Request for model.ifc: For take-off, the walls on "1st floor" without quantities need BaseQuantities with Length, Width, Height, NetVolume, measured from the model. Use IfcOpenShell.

First a look at what the model holds.

```python
import ifcopenshell
import ifcopenshell.util.element
import ifcopenshell.util.unit

model = ifcopenshell.open("model.ifc")
print(model.schema)
for unit_type in ("LENGTHUNIT", "AREAUNIT", "VOLUMEUNIT"):
    print(unit_type, ifcopenshell.util.unit.calculate_unit_scale(model, unit_type))
storey = next(s for s in model.by_type("IfcBuildingStorey") if s.Name == "1st floor")
walls = [e for e in ifcopenshell.util.element.get_decomposition(storey) if e.is_a("IfcWall")]
for e in sorted(walls, key=lambda e: e.id()):
    print(e.id(), e.is_a(), e.Name, list(ifcopenshell.util.element.get_psets(e, qtos_only=True)), sep=" | ")
```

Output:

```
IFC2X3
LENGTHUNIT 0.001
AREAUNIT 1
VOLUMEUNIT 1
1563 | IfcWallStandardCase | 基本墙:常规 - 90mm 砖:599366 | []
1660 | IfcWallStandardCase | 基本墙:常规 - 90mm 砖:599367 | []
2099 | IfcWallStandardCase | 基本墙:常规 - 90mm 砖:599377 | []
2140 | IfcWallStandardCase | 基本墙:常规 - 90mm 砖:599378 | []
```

```python
import ifcopenshell
import ifcopenshell.api.pset
import ifcopenshell.geom
import ifcopenshell.util.element
import ifcopenshell.util.shape
import ifcopenshell.util.unit

model = ifcopenshell.open("model.ifc")
unit_scale = ifcopenshell.util.unit.calculate_unit_scale(model)
volume_scale = ifcopenshell.util.unit.calculate_unit_scale(model, "VOLUMEUNIT")
settings = ifcopenshell.geom.settings()

storey = next(s for s in model.by_type("IfcBuildingStorey") if s.Name == "1st floor")
walls = [e for e in ifcopenshell.util.element.get_decomposition(storey) if e.is_a("IfcWall")]

for e in sorted(walls, key=lambda e: e.id()):
    if ifcopenshell.util.element.get_psets(e, qtos_only=True, should_inherit=False):
        continue
    # Geometry comes back in metres, in the element's own axes.
    shape = ifcopenshell.geom.create_shape(settings, e)
    values = {
        "Length": ifcopenshell.util.shape.get_x(shape.geometry) / unit_scale,
        "Width": ifcopenshell.util.shape.get_y(shape.geometry) / unit_scale,
        "Height": ifcopenshell.util.shape.get_z(shape.geometry) / unit_scale,
        "NetVolume": ifcopenshell.util.shape.get_volume(shape.geometry) / volume_scale,
    }
    qto = ifcopenshell.api.pset.add_qto(model, product=e, name="BaseQuantities")
    ifcopenshell.api.pset.edit_qto(model, qto=qto, properties=values)
    print(e.id(), {k: round(v, 3) for k, v in values.items()})

model.write("model_edited.ifc")
```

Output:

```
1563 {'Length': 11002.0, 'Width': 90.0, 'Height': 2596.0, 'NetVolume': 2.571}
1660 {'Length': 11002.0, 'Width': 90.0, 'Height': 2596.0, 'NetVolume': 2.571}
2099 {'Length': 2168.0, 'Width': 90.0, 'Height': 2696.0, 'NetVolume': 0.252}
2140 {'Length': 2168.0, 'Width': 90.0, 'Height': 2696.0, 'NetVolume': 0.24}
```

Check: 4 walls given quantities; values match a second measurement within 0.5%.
